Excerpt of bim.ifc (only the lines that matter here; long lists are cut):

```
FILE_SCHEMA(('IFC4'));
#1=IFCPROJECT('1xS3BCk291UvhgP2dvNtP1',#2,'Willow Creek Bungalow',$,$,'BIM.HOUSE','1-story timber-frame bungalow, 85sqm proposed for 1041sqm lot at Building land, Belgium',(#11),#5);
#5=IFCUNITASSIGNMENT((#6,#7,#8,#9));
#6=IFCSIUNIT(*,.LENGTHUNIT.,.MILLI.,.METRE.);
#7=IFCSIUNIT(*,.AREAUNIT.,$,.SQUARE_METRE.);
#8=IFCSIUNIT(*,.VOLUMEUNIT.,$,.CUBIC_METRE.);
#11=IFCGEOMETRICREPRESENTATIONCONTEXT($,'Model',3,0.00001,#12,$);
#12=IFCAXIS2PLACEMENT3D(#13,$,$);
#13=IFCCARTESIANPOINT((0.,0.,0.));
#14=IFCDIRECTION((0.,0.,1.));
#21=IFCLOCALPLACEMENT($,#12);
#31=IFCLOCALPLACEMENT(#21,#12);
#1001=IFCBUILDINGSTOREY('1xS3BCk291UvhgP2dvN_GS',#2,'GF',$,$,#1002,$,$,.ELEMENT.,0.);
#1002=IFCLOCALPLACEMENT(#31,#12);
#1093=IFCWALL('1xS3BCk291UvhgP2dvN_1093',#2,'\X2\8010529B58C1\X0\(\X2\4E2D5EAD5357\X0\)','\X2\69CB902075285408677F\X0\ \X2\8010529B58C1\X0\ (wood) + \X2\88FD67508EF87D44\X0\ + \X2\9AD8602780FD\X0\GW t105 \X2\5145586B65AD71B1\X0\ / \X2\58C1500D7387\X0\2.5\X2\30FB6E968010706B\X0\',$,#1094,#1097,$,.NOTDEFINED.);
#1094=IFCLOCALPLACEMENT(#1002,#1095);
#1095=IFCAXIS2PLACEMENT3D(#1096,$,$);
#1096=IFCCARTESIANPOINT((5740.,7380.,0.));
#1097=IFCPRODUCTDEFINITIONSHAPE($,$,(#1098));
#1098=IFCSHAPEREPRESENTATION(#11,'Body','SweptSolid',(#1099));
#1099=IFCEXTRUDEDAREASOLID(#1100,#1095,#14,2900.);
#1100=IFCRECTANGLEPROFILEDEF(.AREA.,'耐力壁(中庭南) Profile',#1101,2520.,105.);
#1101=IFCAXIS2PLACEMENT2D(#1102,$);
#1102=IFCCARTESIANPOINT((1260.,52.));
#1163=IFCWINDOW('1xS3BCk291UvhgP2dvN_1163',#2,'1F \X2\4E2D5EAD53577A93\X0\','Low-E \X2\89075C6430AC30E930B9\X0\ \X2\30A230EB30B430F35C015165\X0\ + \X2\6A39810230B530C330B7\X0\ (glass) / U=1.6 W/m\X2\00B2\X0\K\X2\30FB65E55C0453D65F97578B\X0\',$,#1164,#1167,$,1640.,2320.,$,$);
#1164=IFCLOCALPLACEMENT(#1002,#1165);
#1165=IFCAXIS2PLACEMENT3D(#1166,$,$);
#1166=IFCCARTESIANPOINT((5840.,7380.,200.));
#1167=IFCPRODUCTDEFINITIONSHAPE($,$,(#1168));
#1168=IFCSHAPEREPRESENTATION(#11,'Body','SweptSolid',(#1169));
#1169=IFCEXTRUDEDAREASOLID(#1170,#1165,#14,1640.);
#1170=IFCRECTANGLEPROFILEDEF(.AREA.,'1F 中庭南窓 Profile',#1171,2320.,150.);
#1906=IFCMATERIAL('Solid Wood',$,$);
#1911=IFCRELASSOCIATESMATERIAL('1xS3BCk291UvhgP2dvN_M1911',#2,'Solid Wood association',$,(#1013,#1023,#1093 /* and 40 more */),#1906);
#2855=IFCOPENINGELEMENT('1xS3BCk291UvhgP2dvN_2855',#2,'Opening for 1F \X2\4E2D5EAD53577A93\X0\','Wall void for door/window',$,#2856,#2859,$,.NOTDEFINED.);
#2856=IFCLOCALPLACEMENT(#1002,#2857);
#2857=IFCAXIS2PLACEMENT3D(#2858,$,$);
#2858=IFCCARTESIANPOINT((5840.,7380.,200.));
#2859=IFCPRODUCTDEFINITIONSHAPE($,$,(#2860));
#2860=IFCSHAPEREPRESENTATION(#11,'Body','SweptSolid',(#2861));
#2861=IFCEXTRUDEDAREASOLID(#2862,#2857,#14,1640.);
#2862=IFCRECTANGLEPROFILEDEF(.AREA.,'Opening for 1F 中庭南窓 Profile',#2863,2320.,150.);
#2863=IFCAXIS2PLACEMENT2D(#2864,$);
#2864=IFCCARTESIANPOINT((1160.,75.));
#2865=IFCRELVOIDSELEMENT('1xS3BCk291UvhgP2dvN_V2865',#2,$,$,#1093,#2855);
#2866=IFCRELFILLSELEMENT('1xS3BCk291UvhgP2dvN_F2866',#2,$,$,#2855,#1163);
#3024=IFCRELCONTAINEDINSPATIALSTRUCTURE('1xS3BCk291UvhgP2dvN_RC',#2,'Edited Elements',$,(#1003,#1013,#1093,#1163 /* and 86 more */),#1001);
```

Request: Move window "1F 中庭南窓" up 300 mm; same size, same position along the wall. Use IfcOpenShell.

```python
import numpy as np
import ifcopenshell
import ifcopenshell.api.geometry
import ifcopenshell.util.placement
import ifcopenshell.util.unit

model = ifcopenshell.open("bim.ifc")
unit_scale = ifcopenshell.util.unit.calculate_unit_scale(model)

window = model.by_guid("1xS3BCk291UvhgP2dvN_1163")
opening = window.FillsVoids[0].RelatingOpeningElement
dz = 0.3 / unit_scale

shift = np.array([0.0, 0.0, dz])
# The window is not placed relative to its opening, so move both.
for product in (opening, window):
    matrix = ifcopenshell.util.placement.get_local_placement(product.ObjectPlacement)
    matrix[:3, 3] += shift
    ifcopenshell.api.geometry.edit_object_placement(model, product=product, matrix=matrix, is_si=False)

print(f"moved by {dz * unit_scale:+.3f} m")

model.write("bim-out.ifc")
```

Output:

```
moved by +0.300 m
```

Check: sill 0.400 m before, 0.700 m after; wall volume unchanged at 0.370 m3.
